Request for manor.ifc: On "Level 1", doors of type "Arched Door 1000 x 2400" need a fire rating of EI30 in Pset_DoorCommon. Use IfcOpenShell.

First a look at what the model holds.

```python
import ifcopenshell
import ifcopenshell.util.element

model = ifcopenshell.open("manor.ifc")
print(model.schema)
storey = next(s for s in model.by_type("IfcBuildingStorey") if s.Name == "Level 1")
doors = [e for e in ifcopenshell.util.element.get_decomposition(storey) if e.is_a("IfcDoor")]
seen = {}
for e in doors:
    element_type = ifcopenshell.util.element.get_type(e)
    key = (element_type.Name if element_type != e and element_type else None, ifcopenshell.util.element.get_pset(e, "Pset_DoorCommon", "FireRating"))
    seen[key] = seen.get(key, 0) + 1
for (name, value), count in sorted(seen.items(), key=str):
    print(count, "x", name, "|", value)
```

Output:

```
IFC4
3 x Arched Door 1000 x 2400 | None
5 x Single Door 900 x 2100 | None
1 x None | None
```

```python
import ifcopenshell
import ifcopenshell.api.pset
import ifcopenshell.util.element

model = ifcopenshell.open("manor.ifc")

storey = next(s for s in model.by_type("IfcBuildingStorey") if s.Name == "Level 1")
doors = [e for e in ifcopenshell.util.element.get_decomposition(storey) if e.is_a("IfcDoor")]

count = 0
for e in doors:
    element_type = ifcopenshell.util.element.get_type(e)
    if element_type in (None, e) or element_type.Name != "Arched Door 1000 x 2400":
        continue
    # add_pset returns the element's existing set when there is one.
    pset = ifcopenshell.api.pset.add_pset(model, product=e, name="Pset_DoorCommon")
    ifcopenshell.api.pset.edit_pset(model, pset=pset, properties={"FireRating": "EI30"})
    count += 1

print(count, "doors updated")

model.write("manor_updated.ifc")
```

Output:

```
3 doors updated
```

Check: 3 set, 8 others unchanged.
